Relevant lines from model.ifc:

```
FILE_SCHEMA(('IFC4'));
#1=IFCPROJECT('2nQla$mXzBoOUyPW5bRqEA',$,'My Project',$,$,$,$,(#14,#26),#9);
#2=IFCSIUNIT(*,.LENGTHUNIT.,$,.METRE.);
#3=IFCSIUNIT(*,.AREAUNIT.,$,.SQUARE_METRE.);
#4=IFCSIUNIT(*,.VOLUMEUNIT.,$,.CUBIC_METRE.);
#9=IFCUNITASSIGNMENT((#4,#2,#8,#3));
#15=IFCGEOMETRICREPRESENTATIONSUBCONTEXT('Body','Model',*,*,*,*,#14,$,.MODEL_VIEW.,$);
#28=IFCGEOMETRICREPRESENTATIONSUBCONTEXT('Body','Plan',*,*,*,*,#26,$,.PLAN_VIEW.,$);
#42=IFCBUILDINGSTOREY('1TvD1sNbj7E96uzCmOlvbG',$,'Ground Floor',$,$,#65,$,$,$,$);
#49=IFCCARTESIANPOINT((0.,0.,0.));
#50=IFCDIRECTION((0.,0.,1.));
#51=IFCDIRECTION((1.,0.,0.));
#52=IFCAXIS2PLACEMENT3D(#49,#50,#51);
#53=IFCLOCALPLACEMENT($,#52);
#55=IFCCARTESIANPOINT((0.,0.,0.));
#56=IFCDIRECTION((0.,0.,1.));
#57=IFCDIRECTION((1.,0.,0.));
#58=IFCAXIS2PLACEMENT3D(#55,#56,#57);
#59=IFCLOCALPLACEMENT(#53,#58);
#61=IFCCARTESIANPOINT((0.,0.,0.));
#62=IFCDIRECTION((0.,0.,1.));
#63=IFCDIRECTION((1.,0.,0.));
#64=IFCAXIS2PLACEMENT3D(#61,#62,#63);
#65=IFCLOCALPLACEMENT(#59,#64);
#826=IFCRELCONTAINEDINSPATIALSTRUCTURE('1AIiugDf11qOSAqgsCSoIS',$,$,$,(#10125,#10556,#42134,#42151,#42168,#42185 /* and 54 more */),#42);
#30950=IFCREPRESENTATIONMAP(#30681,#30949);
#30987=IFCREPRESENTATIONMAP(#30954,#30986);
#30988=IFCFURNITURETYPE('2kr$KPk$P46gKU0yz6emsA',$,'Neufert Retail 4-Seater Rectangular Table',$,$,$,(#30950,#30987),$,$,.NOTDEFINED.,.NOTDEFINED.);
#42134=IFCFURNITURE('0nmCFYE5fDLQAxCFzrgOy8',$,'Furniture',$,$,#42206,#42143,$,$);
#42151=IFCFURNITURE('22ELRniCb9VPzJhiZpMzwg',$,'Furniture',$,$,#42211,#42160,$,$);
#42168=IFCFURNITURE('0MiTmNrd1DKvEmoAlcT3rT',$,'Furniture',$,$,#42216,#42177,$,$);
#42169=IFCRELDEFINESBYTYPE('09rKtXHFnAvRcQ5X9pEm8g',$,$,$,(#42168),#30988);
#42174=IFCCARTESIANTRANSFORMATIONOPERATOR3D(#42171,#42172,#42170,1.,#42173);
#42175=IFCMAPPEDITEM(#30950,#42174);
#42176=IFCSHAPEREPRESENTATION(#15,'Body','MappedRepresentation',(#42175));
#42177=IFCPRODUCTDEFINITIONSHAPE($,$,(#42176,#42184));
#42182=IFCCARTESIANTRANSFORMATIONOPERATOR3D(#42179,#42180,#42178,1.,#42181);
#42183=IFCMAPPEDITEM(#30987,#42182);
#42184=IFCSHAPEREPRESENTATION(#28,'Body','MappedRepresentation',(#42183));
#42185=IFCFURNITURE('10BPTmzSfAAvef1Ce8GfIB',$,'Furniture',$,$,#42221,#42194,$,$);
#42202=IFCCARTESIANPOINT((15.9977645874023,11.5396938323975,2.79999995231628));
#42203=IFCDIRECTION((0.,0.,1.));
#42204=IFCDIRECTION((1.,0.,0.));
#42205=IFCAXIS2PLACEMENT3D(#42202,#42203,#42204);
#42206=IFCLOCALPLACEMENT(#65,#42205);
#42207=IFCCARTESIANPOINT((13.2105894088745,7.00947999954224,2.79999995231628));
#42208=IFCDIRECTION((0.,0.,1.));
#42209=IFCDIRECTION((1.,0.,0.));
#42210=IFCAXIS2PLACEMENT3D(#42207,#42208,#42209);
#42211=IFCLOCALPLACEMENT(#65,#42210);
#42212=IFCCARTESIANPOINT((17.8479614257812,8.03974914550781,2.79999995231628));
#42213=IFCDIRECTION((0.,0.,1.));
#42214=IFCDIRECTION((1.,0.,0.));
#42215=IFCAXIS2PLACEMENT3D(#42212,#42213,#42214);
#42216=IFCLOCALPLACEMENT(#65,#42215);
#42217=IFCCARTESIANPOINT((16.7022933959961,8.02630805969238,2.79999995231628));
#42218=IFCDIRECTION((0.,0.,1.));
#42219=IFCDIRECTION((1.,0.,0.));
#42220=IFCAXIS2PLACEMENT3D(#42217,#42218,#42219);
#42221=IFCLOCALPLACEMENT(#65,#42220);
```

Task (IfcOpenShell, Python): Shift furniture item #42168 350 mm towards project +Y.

```python
import ifcopenshell
import ifcopenshell.api.geometry
import ifcopenshell.util.placement

model = ifcopenshell.open("model.ifc")

item = model.by_guid("0MiTmNrd1DKvEmoAlcT3rT")
matrix = ifcopenshell.util.placement.get_local_placement(item.ObjectPlacement)
matrix[1, 3] += 0.35
ifcopenshell.api.geometry.edit_object_placement(model, product=item, matrix=matrix, is_si=False)

print(ifcopenshell.util.placement.get_local_placement(item.ObjectPlacement).round(3) + 0.0)

model.write("model_edited.ifc")
```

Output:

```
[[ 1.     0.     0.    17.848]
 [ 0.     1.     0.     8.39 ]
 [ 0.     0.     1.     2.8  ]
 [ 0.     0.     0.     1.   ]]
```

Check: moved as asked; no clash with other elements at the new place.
